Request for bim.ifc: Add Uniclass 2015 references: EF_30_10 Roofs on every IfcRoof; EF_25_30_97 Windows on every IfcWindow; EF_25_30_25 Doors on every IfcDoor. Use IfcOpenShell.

First a look at what the model holds.

```python
import ifcopenshell

model = ifcopenshell.open("bim.ifc")
print(model.schema)
print("classifications:", [c.Name for c in model.by_type("IfcClassification")])
for ifc_class in ("IfcDoor", "IfcRoof", "IfcStair", "IfcWall", "IfcWindow"):
    print(ifc_class, len(model.by_type(ifc_class)))
```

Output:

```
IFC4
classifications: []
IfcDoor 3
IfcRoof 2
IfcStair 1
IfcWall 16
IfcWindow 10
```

```python
import ifcopenshell
import ifcopenshell.api.classification

model = ifcopenshell.open("bim.ifc")

system = ifcopenshell.api.classification.add_classification(model, classification="Uniclass 2015")

codes = {
    "IfcRoof": ("EF_30_10", "Roofs"),
    "IfcWindow": ("EF_25_30_97", "Windows"),
    "IfcDoor": ("EF_25_30_25", "Doors"),
}
for ifc_class, (code, name) in codes.items():
    products = model.by_type(ifc_class)
    ifcopenshell.api.classification.add_reference(
        model, products=products, classification=system, identification=code, name=name
    )
    print(code, len(products))

model.write("bim-out.ifc")
```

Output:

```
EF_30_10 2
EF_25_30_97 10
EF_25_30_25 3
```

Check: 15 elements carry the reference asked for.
